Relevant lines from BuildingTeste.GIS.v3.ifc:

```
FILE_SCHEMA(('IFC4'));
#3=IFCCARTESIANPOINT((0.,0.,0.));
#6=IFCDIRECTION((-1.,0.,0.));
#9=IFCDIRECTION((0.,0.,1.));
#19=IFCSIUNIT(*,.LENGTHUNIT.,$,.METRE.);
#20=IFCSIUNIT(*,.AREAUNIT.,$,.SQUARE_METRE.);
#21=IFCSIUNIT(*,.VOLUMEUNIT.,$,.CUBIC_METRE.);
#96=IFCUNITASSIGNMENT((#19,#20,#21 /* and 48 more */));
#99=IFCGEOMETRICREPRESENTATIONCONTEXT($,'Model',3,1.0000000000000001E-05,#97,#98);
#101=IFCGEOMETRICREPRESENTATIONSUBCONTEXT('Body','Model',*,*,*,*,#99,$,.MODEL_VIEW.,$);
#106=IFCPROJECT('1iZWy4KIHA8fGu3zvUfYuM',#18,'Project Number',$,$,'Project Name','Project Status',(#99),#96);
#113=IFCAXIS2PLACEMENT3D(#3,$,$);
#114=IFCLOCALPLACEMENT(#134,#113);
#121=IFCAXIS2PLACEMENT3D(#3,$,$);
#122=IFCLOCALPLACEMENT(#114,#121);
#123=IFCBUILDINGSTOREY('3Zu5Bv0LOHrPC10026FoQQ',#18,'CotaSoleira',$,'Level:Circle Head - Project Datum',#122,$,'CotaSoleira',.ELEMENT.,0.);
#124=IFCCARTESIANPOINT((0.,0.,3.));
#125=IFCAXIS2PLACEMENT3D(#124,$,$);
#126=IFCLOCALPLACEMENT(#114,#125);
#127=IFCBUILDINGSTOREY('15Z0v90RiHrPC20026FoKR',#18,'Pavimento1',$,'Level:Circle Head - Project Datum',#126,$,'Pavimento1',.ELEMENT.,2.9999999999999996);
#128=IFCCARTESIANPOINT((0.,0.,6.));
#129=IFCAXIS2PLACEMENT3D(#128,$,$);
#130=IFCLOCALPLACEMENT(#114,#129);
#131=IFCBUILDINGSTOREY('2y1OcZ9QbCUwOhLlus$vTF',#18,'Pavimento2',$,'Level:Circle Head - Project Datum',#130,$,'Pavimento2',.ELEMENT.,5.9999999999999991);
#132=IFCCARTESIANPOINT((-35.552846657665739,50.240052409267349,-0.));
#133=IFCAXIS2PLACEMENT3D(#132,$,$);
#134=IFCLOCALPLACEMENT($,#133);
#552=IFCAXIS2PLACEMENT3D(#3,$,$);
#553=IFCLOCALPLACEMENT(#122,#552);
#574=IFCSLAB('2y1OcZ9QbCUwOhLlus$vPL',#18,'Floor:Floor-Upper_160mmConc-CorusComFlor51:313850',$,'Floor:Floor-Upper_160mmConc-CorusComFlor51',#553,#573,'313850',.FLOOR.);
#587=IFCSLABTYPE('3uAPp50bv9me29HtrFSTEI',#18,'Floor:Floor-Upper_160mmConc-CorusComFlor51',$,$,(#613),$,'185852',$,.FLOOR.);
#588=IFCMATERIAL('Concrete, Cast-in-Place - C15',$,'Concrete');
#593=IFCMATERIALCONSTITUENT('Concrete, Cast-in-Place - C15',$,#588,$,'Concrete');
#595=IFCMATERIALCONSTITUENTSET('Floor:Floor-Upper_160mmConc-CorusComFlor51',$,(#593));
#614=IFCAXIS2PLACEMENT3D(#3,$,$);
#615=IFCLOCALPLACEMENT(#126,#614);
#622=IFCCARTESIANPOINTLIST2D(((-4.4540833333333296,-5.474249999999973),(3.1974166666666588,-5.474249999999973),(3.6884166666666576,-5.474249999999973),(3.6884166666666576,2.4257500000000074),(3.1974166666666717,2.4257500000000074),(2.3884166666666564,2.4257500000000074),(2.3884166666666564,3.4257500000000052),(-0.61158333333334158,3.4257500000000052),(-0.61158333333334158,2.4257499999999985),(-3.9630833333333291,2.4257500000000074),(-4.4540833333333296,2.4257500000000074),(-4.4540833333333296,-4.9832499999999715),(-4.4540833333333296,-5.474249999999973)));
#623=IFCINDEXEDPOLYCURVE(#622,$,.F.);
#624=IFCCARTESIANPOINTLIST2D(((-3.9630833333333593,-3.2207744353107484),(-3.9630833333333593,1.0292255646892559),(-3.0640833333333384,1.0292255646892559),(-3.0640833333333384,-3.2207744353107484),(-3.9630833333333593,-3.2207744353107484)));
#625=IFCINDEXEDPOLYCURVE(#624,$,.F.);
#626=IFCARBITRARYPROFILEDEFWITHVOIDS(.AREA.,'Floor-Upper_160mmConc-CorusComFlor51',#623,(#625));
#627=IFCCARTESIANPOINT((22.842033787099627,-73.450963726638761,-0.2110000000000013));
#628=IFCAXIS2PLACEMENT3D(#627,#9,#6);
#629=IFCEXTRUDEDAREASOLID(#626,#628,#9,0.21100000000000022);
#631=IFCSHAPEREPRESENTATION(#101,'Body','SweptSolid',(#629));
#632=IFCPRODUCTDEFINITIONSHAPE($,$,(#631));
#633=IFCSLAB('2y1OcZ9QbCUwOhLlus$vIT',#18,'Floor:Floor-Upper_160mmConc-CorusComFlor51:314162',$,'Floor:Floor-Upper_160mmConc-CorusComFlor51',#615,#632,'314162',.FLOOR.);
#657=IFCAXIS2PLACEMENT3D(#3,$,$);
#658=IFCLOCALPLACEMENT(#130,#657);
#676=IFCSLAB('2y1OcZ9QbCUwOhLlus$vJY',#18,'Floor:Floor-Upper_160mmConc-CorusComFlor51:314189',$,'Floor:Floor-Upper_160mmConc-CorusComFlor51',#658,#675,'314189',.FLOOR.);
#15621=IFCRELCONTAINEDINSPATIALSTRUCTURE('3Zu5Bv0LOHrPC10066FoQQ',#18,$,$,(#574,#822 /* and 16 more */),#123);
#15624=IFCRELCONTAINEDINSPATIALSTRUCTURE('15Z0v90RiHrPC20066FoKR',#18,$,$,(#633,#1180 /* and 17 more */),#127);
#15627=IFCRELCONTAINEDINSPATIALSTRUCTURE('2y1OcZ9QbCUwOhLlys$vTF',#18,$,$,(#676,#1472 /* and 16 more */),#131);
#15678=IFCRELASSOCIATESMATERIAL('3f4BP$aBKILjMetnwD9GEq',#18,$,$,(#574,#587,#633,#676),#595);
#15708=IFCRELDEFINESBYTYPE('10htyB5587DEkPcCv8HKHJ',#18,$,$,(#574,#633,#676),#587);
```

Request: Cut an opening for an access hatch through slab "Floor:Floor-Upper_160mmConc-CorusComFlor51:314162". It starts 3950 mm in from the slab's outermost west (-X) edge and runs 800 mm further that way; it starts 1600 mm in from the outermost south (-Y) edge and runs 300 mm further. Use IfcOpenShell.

```python
import numpy as np
import ifcopenshell
import ifcopenshell.api.feature
import ifcopenshell.api.geometry
import ifcopenshell.api.root
import ifcopenshell.geom
import ifcopenshell.util.placement
import ifcopenshell.util.representation
import ifcopenshell.util.shape
import ifcopenshell.util.unit

model = ifcopenshell.open("BuildingTeste.GIS.v3.ifc")
unit_scale = ifcopenshell.util.unit.calculate_unit_scale(model)
settings = ifcopenshell.geom.settings()


def volume(element):
    """Net volume in cubic metres, openings subtracted."""
    shape = ifcopenshell.geom.create_shape(settings, element)
    return ifcopenshell.util.shape.get_volume(shape.geometry)


slab = model.by_guid("2y1OcZ9QbCUwOhLlus$vIT")
before = volume(slab)

# Extent in the slab's own axes, in metres. The edges named are its -X and -Y sides.
slab_shape = ifcopenshell.geom.create_shape(settings, slab)
vertices = ifcopenshell.util.shape.get_vertices(slab_shape.geometry)
x_min, y_min, bottom = vertices.min(axis=0)
top = vertices[:, 2].max()

opening = ifcopenshell.api.root.create_entity(model, ifc_class="IfcOpeningElement", name="Access hatch opening", predefined_type="OPENING")
context = ifcopenshell.util.representation.get_context(model, "Model", "Body", "MODEL_VIEW")
width, depth = 0.8, 0.3
outline = [(0.0, 0.0), (width, 0.0), (width, depth), (0.0, depth), (0.0, 0.0)]
# Overshoot both faces by 50 mm so the cut is clean.
shape = ifcopenshell.api.geometry.add_slab_representation(
    model, context=context, depth=top - bottom + 0.1, polyline=outline
)
ifcopenshell.api.geometry.assign_representation(model, product=opening, representation=shape)

matrix = ifcopenshell.util.placement.get_local_placement(slab.ObjectPlacement)
matrix[:, 3] = matrix @ np.append(np.array([x_min + 3.95, y_min + 1.6, bottom - 0.05]) / unit_scale, 1.0)
ifcopenshell.api.geometry.edit_object_placement(model, product=opening, matrix=matrix, is_si=False)
ifcopenshell.api.feature.add_feature(model, feature=opening, element=slab)

after = volume(slab)

print(f"slab volume {before:.3f} -> {after:.3f} m3")

model.write("BuildingTeste.GIS.v3_v2.ifc")
```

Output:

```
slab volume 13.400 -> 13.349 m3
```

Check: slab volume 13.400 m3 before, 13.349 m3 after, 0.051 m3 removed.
